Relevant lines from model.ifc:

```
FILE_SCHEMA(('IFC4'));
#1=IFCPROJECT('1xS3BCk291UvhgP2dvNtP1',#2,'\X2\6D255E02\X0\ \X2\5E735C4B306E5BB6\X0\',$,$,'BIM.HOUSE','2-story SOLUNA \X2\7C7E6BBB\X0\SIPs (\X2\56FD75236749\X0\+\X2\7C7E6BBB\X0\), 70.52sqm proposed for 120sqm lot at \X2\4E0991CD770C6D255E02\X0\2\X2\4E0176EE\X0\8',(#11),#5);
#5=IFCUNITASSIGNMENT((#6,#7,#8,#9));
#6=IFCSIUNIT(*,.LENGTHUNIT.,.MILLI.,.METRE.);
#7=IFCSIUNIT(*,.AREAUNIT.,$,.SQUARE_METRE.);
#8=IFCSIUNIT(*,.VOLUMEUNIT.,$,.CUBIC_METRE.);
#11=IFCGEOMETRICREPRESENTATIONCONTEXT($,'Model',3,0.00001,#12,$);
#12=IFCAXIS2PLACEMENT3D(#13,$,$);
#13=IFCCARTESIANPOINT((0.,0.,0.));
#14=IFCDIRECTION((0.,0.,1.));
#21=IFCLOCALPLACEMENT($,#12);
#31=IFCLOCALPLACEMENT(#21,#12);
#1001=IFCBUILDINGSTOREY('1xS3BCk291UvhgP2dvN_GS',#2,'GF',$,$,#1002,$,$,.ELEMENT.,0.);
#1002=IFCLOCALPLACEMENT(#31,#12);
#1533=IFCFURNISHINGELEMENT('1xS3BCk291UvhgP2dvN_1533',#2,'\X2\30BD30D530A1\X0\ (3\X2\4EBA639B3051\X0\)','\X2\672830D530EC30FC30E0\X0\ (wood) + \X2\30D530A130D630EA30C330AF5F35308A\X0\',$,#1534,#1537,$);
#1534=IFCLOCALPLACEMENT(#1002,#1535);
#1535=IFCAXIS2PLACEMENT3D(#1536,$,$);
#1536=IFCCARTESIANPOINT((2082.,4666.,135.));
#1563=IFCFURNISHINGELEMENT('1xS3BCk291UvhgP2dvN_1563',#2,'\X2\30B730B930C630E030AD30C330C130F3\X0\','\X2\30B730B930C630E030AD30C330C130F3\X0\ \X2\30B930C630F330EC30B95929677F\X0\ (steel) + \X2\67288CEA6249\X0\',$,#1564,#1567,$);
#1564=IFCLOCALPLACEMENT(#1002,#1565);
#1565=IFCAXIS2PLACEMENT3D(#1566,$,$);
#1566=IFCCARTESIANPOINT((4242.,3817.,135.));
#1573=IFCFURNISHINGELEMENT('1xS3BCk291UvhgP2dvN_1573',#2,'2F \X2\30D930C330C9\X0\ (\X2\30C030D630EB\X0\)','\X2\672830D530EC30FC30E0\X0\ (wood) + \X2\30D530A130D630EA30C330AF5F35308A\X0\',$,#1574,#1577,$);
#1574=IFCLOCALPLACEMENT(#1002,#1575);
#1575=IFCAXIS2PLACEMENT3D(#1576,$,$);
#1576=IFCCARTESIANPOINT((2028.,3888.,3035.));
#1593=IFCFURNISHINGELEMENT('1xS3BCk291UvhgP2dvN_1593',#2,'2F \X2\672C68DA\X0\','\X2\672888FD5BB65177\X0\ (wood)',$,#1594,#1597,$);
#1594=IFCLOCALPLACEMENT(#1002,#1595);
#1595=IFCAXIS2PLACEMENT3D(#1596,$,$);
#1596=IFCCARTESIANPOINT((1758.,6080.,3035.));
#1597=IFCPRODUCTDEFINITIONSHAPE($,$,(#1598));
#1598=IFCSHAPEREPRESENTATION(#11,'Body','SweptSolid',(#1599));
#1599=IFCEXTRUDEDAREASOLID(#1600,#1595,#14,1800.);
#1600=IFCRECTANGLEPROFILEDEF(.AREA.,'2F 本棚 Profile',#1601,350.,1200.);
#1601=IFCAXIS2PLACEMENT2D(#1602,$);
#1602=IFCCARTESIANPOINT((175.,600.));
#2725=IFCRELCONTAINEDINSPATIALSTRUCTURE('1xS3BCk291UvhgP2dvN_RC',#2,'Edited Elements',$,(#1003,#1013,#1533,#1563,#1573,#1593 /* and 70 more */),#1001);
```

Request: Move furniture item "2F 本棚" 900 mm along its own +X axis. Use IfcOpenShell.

```python
import ifcopenshell
import ifcopenshell.api.geometry
import ifcopenshell.util.placement

model = ifcopenshell.open("model.ifc")

item = model.by_guid("1xS3BCk291UvhgP2dvN_1593")
matrix = ifcopenshell.util.placement.get_local_placement(item.ObjectPlacement)
matrix[:3, 3] += matrix[:3, 0] * 900.0
ifcopenshell.api.geometry.edit_object_placement(model, product=item, matrix=matrix, is_si=False)

print(ifcopenshell.util.placement.get_local_placement(item.ObjectPlacement).round(3) + 0.0)

model.write("model_updated.ifc")
```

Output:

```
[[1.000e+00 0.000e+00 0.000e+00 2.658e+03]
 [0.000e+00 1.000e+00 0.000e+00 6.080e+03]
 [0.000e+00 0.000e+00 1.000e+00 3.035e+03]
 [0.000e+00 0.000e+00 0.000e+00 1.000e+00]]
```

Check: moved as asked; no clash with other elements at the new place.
